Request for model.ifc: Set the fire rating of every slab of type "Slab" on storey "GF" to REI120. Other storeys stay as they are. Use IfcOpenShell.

First a look at what the model holds.

```python
import ifcopenshell
import ifcopenshell.util.element

model = ifcopenshell.open("model.ifc")
print(model.schema)
storey = next(s for s in model.by_type("IfcBuildingStorey") if s.Name == "GF")
slabs = [e for e in ifcopenshell.util.element.get_decomposition(storey) if e.is_a("IfcSlab")]
seen = {}
for e in slabs:
    element_type = ifcopenshell.util.element.get_type(e)
    key = (element_type.Name if element_type != e and element_type else None, ifcopenshell.util.element.get_pset(e, "Pset_SlabCommon", "FireRating"))
    seen[key] = seen.get(key, 0) + 1
for (name, value), count in sorted(seen.items(), key=str):
    print(count, "x", name, "|", value)
```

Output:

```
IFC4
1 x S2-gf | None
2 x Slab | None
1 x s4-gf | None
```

```python
import ifcopenshell
import ifcopenshell.api.pset
import ifcopenshell.util.element

model = ifcopenshell.open("model.ifc")

storey = next(s for s in model.by_type("IfcBuildingStorey") if s.Name == "GF")
slabs = [e for e in ifcopenshell.util.element.get_decomposition(storey) if e.is_a("IfcSlab")]

count = 0
for e in slabs:
    element_type = ifcopenshell.util.element.get_type(e)
    if element_type in (None, e) or element_type.Name != "Slab":
        continue
    # add_pset returns the element's existing set when there is one.
    pset = ifcopenshell.api.pset.add_pset(model, product=e, name="Pset_SlabCommon")
    ifcopenshell.api.pset.edit_pset(model, pset=pset, properties={"FireRating": "REI120"})
    count += 1

print(count, "slabs updated")

model.write("model-out.ifc")
```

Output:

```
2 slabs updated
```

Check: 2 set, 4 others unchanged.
